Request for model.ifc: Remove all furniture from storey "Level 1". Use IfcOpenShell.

First a look at what the model holds.

```python
import ifcopenshell
import ifcopenshell.util.element

model = ifcopenshell.open("model.ifc")
print(model.schema)
storey = next(s for s in model.by_type("IfcBuildingStorey") if s.Name == "Level 1")
furniture = [e for e in ifcopenshell.util.element.get_decomposition(storey) if e.is_a("IfcFurnishingElement")]
seen = {}
for e in furniture:
    element_type = ifcopenshell.util.element.get_type(e)
    name = element_type.Name if element_type not in (None, e) else None
    seen[name] = seen.get(name, 0) + 1
for name, count in sorted(seen.items(), key=str):
    print(count, "x", name)
```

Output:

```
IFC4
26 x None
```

```python
import ifcopenshell
import ifcopenshell.api.root
import ifcopenshell.util.element

model = ifcopenshell.open("model.ifc")

storey = next(s for s in model.by_type("IfcBuildingStorey") if s.Name == "Level 1")
furniture = [e for e in ifcopenshell.util.element.get_decomposition(storey) if e.is_a("IfcFurnishingElement")]

for e in furniture:
    ifcopenshell.api.root.remove_product(model, product=e)
print(len(furniture), "removed")

model.write("model-out.ifc")
```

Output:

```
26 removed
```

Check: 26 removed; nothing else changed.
